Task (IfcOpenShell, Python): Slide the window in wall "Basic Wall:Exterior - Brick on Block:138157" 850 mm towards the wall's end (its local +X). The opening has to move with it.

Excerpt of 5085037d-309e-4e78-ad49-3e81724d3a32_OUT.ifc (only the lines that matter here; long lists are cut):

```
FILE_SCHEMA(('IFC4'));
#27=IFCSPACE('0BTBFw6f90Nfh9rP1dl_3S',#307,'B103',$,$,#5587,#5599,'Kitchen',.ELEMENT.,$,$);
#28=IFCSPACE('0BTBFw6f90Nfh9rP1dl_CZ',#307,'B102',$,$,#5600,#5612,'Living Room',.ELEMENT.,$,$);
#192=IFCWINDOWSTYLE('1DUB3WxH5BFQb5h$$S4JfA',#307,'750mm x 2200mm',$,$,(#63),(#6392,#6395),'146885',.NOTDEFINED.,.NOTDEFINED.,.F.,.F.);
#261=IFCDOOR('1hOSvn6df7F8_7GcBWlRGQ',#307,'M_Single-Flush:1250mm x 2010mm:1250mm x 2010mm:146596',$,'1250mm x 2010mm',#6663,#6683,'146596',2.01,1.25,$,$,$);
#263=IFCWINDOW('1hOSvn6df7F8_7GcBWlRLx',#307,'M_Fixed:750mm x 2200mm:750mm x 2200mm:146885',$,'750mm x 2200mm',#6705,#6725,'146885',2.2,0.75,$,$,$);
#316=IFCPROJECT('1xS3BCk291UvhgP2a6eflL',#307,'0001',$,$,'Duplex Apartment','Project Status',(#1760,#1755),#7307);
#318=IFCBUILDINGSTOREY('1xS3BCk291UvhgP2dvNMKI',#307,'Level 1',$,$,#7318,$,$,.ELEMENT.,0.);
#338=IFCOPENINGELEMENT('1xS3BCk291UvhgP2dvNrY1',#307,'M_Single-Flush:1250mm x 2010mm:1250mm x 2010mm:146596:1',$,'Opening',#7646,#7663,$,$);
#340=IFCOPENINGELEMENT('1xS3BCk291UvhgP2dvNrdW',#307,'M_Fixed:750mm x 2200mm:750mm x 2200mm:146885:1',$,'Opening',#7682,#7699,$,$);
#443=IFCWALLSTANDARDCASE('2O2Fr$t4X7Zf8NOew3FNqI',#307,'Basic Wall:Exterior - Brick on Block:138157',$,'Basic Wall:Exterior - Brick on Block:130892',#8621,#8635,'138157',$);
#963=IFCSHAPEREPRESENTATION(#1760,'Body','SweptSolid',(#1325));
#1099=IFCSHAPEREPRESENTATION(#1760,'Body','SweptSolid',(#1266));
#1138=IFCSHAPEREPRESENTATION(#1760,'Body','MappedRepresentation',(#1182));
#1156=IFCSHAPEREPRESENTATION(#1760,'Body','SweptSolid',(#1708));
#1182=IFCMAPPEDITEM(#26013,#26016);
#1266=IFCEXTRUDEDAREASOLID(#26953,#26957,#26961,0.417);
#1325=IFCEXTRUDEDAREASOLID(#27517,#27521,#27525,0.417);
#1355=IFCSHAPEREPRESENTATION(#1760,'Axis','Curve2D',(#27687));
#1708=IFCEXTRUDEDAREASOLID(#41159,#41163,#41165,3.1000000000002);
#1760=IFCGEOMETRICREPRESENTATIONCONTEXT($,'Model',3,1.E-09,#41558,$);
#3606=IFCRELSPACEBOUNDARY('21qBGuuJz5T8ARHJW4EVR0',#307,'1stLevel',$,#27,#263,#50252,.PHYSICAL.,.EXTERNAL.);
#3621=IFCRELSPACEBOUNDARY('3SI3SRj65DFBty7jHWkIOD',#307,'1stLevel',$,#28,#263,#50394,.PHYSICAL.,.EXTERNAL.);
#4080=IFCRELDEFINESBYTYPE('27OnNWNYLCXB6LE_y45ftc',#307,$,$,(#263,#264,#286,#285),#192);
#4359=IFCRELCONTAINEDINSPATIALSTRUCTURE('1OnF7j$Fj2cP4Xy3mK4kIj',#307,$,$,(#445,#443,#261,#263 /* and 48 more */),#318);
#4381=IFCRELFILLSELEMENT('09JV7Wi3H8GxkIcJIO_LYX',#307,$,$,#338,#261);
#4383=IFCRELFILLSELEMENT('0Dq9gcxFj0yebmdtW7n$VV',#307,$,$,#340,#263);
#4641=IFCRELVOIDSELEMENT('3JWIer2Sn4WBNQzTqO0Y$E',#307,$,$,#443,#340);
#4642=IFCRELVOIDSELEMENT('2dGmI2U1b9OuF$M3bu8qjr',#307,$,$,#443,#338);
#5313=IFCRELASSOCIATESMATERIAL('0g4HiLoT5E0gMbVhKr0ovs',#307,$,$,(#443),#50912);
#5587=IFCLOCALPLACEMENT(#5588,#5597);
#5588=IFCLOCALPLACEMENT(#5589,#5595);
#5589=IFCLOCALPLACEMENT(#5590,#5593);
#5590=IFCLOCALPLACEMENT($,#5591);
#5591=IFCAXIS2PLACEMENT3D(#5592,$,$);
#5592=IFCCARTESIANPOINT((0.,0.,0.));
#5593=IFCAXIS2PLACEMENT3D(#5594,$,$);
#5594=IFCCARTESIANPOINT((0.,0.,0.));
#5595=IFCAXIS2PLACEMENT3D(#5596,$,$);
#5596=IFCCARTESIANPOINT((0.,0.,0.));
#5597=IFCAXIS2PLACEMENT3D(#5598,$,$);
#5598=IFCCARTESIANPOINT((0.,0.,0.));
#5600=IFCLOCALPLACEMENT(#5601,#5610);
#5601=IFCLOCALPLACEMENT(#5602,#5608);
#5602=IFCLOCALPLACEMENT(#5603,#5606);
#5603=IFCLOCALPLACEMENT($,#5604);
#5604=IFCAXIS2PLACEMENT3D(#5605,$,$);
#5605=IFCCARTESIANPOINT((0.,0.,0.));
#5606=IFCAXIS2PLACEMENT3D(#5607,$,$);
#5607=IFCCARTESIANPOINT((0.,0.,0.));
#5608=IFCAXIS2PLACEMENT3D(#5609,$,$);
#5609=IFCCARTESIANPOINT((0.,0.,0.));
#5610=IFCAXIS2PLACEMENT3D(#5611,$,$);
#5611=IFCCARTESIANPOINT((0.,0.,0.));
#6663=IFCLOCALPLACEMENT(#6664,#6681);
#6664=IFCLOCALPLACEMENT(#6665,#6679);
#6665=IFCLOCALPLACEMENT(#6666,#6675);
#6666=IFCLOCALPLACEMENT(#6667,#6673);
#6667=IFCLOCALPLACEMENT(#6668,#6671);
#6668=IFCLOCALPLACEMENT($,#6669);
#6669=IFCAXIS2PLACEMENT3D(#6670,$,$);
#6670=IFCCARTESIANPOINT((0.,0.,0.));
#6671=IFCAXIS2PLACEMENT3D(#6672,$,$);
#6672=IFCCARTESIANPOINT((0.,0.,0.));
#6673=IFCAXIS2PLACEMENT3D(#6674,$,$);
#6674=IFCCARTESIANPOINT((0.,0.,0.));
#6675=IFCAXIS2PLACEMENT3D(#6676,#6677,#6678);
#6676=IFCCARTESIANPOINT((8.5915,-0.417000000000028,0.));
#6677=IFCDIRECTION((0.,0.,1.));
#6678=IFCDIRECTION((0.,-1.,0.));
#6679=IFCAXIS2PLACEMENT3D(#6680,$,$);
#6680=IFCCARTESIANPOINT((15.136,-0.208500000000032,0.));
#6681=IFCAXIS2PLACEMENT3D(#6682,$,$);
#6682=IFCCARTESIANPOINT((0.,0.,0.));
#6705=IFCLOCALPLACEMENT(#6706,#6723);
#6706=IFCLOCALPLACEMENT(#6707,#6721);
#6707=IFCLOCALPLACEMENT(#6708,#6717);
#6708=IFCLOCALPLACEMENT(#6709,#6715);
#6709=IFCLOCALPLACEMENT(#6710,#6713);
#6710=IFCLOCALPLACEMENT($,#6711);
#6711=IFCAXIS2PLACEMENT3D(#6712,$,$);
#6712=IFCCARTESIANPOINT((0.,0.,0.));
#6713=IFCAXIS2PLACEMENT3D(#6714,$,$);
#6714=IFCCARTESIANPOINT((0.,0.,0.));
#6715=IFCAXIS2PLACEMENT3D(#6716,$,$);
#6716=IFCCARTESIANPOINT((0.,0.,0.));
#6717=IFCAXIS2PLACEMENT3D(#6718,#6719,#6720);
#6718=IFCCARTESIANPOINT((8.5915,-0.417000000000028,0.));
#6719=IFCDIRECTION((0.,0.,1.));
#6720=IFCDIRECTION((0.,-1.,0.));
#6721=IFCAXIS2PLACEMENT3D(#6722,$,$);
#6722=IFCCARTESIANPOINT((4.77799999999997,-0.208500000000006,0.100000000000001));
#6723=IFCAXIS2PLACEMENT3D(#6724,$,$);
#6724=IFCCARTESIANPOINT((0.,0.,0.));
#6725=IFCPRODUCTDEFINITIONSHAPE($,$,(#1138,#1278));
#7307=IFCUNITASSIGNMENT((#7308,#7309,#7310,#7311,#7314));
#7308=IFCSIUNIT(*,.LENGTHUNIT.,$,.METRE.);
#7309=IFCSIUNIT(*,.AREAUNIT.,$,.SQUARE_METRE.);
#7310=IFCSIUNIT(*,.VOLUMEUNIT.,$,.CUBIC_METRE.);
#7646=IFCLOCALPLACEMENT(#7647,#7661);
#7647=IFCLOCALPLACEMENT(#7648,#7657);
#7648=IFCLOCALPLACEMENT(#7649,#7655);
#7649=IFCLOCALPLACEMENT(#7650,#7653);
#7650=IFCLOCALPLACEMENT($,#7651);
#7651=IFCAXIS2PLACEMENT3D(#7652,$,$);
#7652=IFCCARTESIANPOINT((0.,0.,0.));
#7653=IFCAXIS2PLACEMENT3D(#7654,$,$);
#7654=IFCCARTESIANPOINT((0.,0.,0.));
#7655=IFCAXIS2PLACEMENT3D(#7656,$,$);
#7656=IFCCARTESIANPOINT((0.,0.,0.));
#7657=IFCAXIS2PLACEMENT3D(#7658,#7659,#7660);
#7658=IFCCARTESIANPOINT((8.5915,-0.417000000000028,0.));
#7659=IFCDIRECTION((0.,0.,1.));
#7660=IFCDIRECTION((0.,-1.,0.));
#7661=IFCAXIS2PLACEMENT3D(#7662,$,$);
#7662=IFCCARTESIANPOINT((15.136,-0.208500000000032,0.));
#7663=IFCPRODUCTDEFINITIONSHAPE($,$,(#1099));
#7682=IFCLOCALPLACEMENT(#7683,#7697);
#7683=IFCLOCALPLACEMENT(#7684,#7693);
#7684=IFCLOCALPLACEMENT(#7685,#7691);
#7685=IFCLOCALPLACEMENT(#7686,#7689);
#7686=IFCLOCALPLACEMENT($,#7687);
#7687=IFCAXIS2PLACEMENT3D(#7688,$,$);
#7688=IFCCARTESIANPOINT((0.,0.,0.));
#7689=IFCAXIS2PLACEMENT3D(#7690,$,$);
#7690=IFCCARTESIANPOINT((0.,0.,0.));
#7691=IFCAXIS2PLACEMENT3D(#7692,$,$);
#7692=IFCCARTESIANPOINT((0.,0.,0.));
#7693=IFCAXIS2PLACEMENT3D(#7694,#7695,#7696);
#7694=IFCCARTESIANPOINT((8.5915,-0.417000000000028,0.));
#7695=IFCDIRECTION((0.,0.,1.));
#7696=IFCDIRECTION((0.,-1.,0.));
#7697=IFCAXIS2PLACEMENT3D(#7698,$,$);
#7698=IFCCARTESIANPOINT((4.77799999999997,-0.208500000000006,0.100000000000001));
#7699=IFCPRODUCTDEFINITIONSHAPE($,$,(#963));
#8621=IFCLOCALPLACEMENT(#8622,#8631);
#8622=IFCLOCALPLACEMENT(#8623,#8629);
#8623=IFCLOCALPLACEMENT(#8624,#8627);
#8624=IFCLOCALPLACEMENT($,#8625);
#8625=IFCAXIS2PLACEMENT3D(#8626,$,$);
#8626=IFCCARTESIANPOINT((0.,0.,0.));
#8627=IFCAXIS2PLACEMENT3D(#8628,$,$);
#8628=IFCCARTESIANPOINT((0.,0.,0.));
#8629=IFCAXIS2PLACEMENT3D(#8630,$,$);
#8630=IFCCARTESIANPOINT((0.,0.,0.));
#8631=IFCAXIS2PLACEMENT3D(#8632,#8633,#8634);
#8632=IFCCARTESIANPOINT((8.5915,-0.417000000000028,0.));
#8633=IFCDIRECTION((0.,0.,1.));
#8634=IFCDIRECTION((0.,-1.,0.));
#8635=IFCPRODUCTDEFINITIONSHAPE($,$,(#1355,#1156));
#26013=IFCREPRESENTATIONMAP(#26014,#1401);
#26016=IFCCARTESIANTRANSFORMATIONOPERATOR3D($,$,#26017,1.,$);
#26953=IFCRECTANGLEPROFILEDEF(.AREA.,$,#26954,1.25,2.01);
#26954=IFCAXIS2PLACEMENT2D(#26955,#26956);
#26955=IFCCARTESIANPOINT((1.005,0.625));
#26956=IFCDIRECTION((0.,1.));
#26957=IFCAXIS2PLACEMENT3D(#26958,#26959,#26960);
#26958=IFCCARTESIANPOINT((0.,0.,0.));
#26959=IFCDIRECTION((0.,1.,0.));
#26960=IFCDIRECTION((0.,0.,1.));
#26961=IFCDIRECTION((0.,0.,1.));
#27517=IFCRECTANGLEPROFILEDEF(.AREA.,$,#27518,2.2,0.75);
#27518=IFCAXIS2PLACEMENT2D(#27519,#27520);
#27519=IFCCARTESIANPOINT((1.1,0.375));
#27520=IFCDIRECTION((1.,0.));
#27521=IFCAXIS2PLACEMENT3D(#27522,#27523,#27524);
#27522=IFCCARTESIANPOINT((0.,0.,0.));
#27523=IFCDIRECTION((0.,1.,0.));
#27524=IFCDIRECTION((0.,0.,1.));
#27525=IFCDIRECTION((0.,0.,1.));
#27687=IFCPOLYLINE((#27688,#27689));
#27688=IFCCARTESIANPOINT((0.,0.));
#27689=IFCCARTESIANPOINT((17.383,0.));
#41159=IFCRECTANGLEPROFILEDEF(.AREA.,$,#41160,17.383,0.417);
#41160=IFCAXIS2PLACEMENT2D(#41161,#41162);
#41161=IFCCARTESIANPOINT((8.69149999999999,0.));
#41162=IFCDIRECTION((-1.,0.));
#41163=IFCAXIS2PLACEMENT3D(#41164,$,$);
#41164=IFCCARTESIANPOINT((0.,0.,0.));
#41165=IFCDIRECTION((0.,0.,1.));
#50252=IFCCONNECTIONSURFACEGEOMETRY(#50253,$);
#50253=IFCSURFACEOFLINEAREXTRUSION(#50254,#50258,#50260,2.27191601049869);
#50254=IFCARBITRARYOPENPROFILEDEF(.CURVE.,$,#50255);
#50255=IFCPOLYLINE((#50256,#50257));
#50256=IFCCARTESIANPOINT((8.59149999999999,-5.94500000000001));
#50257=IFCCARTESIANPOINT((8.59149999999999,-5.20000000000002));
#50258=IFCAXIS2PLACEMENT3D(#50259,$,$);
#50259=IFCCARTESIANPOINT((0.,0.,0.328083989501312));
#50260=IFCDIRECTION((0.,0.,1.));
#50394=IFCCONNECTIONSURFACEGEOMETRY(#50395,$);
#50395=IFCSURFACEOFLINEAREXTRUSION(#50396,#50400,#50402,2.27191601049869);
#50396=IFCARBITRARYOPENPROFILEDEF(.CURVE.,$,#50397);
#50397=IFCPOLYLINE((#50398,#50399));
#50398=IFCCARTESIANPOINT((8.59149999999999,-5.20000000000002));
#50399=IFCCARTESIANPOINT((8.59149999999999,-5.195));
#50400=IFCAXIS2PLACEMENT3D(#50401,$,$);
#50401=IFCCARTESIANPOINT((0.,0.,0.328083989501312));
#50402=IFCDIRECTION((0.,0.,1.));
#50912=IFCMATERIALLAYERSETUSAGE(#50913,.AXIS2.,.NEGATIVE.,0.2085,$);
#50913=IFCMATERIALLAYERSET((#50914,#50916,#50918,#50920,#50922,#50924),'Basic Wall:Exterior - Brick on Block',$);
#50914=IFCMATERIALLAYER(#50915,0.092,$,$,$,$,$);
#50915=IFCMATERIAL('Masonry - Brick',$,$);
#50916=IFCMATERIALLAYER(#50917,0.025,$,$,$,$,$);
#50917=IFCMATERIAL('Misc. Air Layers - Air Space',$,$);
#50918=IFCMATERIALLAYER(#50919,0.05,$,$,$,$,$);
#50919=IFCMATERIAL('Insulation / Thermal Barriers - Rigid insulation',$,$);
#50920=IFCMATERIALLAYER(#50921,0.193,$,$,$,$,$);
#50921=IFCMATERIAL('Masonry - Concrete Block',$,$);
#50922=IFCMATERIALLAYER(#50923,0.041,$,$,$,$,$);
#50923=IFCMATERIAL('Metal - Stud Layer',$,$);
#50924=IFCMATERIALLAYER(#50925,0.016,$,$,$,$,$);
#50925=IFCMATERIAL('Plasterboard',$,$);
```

```python
import numpy as np
import ifcopenshell
import ifcopenshell.api.geometry
import ifcopenshell.util.placement

model = ifcopenshell.open("5085037d-309e-4e78-ad49-3e81724d3a32_OUT.ifc")

window = model.by_guid("1hOSvn6df7F8_7GcBWlRLx")
opening = window.FillsVoids[0].RelatingOpeningElement
wall = opening.VoidsElements[0].RelatingBuildingElement

wall_matrix = ifcopenshell.util.placement.get_local_placement(wall.ObjectPlacement)
shift = wall_matrix[:3, 0] * 0.85
before = ifcopenshell.util.placement.get_local_placement(window.ObjectPlacement)[:3, 3].copy()

# The window is not placed relative to its opening, so move both.
for product in (opening, window):
    matrix = ifcopenshell.util.placement.get_local_placement(product.ObjectPlacement)
    matrix[:3, 3] += shift
    ifcopenshell.api.geometry.edit_object_placement(model, product=product, matrix=matrix, is_si=False)

# Space boundary surfaces are stored in each space's coordinates; move them too.
for rel in window.ProvidesBoundaries:
    if not rel.ConnectionGeometry:
        continue
    surface = rel.ConnectionGeometry.SurfaceOnRelatingElement
    space_matrix = ifcopenshell.util.placement.get_local_placement(rel.RelatingSpace.ObjectPlacement)
    point = np.array(surface.Position.Location.Coordinates) + space_matrix[:3, :3].T @ shift
    surface.Position = model.createIfcAxis2Placement3D(
        model.createIfcCartesianPoint(point.tolist()), surface.Position.Axis, surface.Position.RefDirection
    )

after = ifcopenshell.util.placement.get_local_placement(window.ObjectPlacement)[:3, 3]
print("window moved by", (after - before).round(3) + 0.0)

model.write("5085037d-309e-4e78-ad49-3e81724d3a32_OUT_edited.ifc")
```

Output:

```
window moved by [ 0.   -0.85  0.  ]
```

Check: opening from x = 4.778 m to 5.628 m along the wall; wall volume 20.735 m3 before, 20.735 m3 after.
